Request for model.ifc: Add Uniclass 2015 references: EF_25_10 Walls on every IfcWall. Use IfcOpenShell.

First a look at what the model holds.

```python
import ifcopenshell

model = ifcopenshell.open("model.ifc")
print(model.schema)
print("classifications:", [c.Name for c in model.by_type("IfcClassification")])
for ifc_class in ("IfcDoor", "IfcRoof", "IfcStair", "IfcWall", "IfcWindow"):
    print(ifc_class, len(model.by_type(ifc_class)))
```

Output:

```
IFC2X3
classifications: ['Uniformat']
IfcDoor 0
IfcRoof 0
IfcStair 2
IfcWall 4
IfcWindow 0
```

```python
import ifcopenshell
import ifcopenshell.api.classification

model = ifcopenshell.open("model.ifc")

# IFC2X3 requires Source and Edition and has no link from the project to the system.
system = model.create_entity("IfcClassification", Source="NBS", Edition="2015", Name="Uniclass 2015")

codes = {
    "IfcWall": ("EF_25_10", "Walls"),
}
for ifc_class, (code, name) in codes.items():
    products = model.by_type(ifc_class)
    ifcopenshell.api.classification.add_reference(
        model, products=products, classification=system, identification=code, name=name
    )
    print(code, len(products))

model.write("model_v2.ifc")
```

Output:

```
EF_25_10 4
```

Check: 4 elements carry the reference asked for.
